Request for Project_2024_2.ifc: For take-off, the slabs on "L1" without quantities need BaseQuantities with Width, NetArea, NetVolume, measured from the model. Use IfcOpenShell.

First a look at what the model holds.

```python
import ifcopenshell
import ifcopenshell.util.element
import ifcopenshell.util.unit

model = ifcopenshell.open("Project_2024_2.ifc")
print(model.schema)
for unit_type in ("LENGTHUNIT", "AREAUNIT", "VOLUMEUNIT"):
    print(unit_type, ifcopenshell.util.unit.calculate_unit_scale(model, unit_type))
storey = next(s for s in model.by_type("IfcBuildingStorey") if s.Name == "L1")
slabs = [e for e in ifcopenshell.util.element.get_decomposition(storey) if e.is_a("IfcSlab")]
for e in sorted(slabs, key=lambda e: e.id()):
    print(e.id(), e.is_a(), e.Name, list(ifcopenshell.util.element.get_psets(e, qtos_only=True)), sep=" | ")
```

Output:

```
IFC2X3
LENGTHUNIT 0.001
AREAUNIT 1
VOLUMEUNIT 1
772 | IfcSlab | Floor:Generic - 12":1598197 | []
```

```python
import ifcopenshell
import ifcopenshell.api.pset
import ifcopenshell.geom
import ifcopenshell.util.element
import ifcopenshell.util.shape
import ifcopenshell.util.unit

model = ifcopenshell.open("Project_2024_2.ifc")
unit_scale = ifcopenshell.util.unit.calculate_unit_scale(model)
area_scale = ifcopenshell.util.unit.calculate_unit_scale(model, "AREAUNIT")
volume_scale = ifcopenshell.util.unit.calculate_unit_scale(model, "VOLUMEUNIT")
settings = ifcopenshell.geom.settings()

storey = next(s for s in model.by_type("IfcBuildingStorey") if s.Name == "L1")
slabs = [e for e in ifcopenshell.util.element.get_decomposition(storey) if e.is_a("IfcSlab")]

for e in sorted(slabs, key=lambda e: e.id()):
    if ifcopenshell.util.element.get_psets(e, qtos_only=True, should_inherit=False):
        continue
    # Geometry comes back in metres, in the element's own axes.
    shape = ifcopenshell.geom.create_shape(settings, e)
    values = {
        "Width": ifcopenshell.util.shape.get_z(shape.geometry) / unit_scale,
        "NetArea": ifcopenshell.util.shape.get_footprint_area(shape.geometry) / area_scale,
        "NetVolume": ifcopenshell.util.shape.get_volume(shape.geometry) / volume_scale,
    }
    qto = ifcopenshell.api.pset.add_qto(model, product=e, name="BaseQuantities")
    ifcopenshell.api.pset.edit_qto(model, qto=qto, properties=values)
    print(e.id(), {k: round(v, 3) for k, v in values.items()})

model.write("Project_2024_2_v2.ifc")
```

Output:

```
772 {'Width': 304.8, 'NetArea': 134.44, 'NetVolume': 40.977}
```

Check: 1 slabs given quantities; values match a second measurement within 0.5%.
